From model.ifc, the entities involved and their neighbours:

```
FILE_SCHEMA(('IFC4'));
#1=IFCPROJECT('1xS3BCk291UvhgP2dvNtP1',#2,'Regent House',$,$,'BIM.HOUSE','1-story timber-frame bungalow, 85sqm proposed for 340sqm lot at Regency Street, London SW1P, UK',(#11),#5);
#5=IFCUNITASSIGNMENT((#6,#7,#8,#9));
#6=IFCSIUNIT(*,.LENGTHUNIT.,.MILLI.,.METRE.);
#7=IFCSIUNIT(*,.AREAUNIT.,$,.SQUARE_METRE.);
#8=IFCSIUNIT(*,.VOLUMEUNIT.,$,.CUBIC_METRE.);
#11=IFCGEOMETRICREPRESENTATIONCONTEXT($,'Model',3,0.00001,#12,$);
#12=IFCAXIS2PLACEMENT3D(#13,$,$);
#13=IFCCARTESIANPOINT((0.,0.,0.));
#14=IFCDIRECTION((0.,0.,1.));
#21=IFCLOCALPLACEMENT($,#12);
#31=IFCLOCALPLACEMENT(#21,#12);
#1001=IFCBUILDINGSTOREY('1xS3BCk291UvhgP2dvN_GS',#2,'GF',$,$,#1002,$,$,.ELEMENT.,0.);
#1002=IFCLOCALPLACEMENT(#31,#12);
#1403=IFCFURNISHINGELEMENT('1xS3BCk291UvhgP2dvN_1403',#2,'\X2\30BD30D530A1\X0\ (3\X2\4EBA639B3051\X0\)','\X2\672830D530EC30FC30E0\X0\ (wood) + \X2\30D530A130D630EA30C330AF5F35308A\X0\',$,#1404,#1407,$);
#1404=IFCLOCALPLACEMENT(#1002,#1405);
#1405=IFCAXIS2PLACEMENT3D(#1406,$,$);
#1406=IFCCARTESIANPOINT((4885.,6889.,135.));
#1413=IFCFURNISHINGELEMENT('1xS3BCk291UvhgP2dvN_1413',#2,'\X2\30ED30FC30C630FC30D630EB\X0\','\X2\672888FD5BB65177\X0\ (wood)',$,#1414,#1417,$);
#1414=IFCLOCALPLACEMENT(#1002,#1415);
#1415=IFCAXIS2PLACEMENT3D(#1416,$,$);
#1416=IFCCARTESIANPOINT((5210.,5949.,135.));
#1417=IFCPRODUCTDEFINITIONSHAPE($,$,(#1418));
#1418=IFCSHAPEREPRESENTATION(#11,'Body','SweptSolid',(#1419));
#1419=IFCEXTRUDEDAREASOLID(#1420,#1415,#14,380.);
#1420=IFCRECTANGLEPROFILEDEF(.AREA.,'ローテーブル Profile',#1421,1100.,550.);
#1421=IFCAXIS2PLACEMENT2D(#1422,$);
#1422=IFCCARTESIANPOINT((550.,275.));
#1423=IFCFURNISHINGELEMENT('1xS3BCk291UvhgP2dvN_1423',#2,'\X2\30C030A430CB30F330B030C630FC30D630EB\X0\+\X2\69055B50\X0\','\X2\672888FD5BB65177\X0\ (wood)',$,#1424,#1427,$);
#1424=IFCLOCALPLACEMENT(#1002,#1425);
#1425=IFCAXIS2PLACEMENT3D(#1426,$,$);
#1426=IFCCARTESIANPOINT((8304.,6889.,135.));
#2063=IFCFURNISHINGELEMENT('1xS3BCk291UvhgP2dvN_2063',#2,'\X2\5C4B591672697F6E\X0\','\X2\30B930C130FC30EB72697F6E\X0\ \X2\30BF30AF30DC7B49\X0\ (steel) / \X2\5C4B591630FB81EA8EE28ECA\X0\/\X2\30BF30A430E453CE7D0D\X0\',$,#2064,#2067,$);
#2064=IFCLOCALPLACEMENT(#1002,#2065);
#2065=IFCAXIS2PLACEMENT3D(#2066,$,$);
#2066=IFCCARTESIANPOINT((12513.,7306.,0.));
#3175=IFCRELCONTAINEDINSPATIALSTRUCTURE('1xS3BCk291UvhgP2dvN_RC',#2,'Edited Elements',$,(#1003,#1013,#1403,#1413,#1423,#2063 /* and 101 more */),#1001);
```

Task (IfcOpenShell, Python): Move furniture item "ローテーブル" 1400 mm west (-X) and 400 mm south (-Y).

```python
import ifcopenshell
import ifcopenshell.api.geometry
import ifcopenshell.util.placement

model = ifcopenshell.open("model.ifc")

item = model.by_guid("1xS3BCk291UvhgP2dvN_1413")
matrix = ifcopenshell.util.placement.get_local_placement(item.ObjectPlacement)
matrix[0, 3] -= 1400.0
matrix[1, 3] -= 400.0
ifcopenshell.api.geometry.edit_object_placement(model, product=item, matrix=matrix, is_si=False)

print(ifcopenshell.util.placement.get_local_placement(item.ObjectPlacement).round(3) + 0.0)

model.write("model_v2.ifc")
```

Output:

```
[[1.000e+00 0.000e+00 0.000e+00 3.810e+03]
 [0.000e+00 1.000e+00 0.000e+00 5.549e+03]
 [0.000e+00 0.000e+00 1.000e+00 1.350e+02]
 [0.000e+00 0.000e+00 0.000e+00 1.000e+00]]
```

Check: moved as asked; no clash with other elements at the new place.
